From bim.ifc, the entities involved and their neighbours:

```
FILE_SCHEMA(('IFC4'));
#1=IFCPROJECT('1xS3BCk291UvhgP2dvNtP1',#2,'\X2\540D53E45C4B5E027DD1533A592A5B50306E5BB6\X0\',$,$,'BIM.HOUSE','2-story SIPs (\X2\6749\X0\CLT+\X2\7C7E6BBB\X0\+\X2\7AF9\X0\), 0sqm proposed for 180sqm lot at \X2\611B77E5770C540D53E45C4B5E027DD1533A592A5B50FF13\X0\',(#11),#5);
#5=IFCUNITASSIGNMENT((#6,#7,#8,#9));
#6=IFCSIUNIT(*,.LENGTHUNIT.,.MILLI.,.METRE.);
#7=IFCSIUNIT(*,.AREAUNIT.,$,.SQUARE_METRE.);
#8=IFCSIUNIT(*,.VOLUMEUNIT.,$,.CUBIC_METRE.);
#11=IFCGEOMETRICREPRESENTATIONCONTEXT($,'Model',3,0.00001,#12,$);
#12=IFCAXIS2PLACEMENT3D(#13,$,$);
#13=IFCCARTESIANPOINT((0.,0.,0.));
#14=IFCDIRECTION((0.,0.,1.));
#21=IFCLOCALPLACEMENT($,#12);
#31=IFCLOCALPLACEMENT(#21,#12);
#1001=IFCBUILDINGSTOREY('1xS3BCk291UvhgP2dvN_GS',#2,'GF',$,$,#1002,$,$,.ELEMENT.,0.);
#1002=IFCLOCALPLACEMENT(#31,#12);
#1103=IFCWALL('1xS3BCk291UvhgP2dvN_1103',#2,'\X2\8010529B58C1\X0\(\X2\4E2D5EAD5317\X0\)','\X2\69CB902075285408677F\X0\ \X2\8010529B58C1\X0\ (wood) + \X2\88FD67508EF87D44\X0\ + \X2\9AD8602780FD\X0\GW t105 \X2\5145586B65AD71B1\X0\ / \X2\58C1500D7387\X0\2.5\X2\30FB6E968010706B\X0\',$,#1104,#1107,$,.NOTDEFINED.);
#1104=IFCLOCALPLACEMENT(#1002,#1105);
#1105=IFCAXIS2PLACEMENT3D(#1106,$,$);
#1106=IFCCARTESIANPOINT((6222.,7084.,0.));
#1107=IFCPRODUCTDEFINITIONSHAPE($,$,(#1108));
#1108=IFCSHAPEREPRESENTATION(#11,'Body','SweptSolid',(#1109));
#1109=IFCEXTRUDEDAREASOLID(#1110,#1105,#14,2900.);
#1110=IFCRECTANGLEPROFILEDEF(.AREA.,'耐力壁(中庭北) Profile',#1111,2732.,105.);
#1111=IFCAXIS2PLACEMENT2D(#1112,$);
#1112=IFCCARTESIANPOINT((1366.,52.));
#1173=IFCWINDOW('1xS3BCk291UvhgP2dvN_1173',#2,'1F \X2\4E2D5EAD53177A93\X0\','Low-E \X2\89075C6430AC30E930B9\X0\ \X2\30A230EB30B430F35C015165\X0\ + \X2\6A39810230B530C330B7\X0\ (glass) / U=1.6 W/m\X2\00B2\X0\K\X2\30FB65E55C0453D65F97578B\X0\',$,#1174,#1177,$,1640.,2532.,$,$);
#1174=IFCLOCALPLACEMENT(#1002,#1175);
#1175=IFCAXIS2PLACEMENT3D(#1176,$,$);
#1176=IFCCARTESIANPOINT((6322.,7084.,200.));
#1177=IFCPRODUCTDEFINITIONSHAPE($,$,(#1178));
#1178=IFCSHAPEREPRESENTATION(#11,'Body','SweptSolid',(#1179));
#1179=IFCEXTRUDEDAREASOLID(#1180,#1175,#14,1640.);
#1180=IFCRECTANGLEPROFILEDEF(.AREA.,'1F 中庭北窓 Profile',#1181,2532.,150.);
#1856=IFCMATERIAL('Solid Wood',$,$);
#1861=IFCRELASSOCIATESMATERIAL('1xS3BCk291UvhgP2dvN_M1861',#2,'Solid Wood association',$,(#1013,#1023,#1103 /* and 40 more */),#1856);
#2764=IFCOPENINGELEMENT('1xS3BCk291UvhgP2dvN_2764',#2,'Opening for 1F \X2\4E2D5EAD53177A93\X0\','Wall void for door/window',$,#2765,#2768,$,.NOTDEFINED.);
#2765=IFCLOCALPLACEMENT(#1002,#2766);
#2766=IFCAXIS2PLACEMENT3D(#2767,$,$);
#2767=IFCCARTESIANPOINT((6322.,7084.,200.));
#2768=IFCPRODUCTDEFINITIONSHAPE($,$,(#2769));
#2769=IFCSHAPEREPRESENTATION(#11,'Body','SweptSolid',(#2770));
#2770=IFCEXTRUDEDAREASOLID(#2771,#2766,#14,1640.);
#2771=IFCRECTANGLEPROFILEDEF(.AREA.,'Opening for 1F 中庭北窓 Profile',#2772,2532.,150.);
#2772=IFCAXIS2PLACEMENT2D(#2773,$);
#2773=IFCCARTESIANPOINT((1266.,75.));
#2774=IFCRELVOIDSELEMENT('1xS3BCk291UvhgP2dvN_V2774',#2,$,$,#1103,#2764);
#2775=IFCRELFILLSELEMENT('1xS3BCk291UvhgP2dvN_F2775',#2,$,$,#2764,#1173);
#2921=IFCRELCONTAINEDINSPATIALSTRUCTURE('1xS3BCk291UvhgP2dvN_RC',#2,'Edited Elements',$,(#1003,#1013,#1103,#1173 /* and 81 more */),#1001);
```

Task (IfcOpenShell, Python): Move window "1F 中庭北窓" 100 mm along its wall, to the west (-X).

```python
import ifcopenshell
import ifcopenshell.api.geometry
import ifcopenshell.util.placement
import ifcopenshell.util.unit

model = ifcopenshell.open("bim.ifc")
unit_scale = ifcopenshell.util.unit.calculate_unit_scale(model)

window = model.by_id(1173)
opening = window.FillsVoids[0].RelatingOpeningElement
wall = opening.VoidsElements[0].RelatingBuildingElement

wall_matrix = ifcopenshell.util.placement.get_local_placement(wall.ObjectPlacement)
shift = wall_matrix[:3, 0] * -0.1 / unit_scale
before = ifcopenshell.util.placement.get_local_placement(window.ObjectPlacement)[:3, 3].copy()

# The window is not placed relative to its opening, so move both.
for product in (opening, window):
    matrix = ifcopenshell.util.placement.get_local_placement(product.ObjectPlacement)
    matrix[:3, 3] += shift
    ifcopenshell.api.geometry.edit_object_placement(model, product=product, matrix=matrix, is_si=False)

after = ifcopenshell.util.placement.get_local_placement(window.ObjectPlacement)[:3, 3]
print("window moved by", (after - before).round(3) + 0.0)

model.write("bim_rev.ifc")
```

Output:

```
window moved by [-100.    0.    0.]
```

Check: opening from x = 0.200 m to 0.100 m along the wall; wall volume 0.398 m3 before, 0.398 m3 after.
